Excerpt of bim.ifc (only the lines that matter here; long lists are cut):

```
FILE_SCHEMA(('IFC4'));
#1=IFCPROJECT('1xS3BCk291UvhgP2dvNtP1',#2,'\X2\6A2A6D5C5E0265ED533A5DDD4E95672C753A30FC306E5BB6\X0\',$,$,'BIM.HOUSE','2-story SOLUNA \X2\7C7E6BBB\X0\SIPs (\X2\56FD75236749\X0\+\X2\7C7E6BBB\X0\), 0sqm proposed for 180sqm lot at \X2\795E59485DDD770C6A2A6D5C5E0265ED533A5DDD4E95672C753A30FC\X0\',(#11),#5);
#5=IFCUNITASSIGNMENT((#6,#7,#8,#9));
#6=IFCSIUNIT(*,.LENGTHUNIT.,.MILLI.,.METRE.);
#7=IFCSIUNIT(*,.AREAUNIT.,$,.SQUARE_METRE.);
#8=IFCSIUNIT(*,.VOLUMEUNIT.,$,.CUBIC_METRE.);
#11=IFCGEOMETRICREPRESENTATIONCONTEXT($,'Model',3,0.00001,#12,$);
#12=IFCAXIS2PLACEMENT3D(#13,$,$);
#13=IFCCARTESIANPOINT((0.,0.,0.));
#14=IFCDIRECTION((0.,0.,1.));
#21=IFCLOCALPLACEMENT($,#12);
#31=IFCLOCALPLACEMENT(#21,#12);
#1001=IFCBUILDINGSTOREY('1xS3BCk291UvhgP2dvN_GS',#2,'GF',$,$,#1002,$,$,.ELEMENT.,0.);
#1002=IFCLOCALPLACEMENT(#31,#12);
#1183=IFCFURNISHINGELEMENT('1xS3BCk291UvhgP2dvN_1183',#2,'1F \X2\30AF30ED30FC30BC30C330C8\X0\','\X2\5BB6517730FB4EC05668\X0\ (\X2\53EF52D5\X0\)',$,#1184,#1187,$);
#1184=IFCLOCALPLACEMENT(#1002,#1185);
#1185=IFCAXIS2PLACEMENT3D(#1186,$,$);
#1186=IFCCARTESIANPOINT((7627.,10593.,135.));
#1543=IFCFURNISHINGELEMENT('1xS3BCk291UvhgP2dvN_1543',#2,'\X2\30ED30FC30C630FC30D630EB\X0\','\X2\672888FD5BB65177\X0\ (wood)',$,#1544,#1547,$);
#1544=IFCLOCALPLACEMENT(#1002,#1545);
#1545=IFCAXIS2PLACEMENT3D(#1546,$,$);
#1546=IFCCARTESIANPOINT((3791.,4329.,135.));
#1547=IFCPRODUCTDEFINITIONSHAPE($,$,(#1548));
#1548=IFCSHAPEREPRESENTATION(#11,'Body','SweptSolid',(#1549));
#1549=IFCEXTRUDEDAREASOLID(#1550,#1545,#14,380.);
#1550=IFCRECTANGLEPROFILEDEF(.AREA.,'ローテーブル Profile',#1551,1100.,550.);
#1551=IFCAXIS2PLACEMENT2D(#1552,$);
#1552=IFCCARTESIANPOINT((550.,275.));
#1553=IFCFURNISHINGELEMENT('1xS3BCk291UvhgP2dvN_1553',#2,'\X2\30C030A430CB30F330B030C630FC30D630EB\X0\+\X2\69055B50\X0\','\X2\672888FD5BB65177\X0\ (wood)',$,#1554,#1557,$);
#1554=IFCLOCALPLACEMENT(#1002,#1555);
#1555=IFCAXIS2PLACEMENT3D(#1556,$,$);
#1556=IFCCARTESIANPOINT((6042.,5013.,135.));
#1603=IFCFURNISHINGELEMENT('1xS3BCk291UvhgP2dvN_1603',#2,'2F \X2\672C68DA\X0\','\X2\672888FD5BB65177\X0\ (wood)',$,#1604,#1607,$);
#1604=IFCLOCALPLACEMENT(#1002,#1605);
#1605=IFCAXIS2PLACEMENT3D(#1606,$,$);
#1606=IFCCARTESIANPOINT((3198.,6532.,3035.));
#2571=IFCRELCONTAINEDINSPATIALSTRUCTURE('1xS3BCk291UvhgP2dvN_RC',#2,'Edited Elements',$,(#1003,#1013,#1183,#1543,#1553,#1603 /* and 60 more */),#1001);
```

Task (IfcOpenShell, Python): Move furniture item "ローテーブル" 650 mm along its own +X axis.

```python
import ifcopenshell
import ifcopenshell.api.geometry
import ifcopenshell.util.placement
import ifcopenshell.util.unit

model = ifcopenshell.open("bim.ifc")
unit_scale = ifcopenshell.util.unit.calculate_unit_scale(model)

item = model.by_guid("1xS3BCk291UvhgP2dvN_1543")
matrix = ifcopenshell.util.placement.get_local_placement(item.ObjectPlacement)
matrix[:3, 3] += matrix[:3, 0] * 0.65 / unit_scale
ifcopenshell.api.geometry.edit_object_placement(model, product=item, matrix=matrix, is_si=False)

print(ifcopenshell.util.placement.get_local_placement(item.ObjectPlacement).round(3) + 0.0)

model.write("bim-out.ifc")
```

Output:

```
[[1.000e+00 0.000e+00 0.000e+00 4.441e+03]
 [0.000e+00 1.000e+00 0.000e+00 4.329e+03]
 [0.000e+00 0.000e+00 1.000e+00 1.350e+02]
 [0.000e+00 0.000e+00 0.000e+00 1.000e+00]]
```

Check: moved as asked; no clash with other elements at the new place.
